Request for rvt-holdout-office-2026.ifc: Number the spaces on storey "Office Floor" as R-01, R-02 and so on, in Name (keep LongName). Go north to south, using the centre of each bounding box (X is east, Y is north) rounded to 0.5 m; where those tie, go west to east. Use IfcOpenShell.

First a look at what the model holds.

```python
import ifcopenshell
import ifcopenshell.util.element
import ifcopenshell.util.placement

model = ifcopenshell.open("rvt-holdout-office-2026.ifc")
print(model.schema)
storey = next(s for s in model.by_type("IfcBuildingStorey") if s.Name == "Office Floor")
spaces = [e for e in ifcopenshell.util.element.get_decomposition(storey) if e.is_a("IfcSpace")]
for e in sorted(spaces, key=lambda e: e.id()):
    origin = ifcopenshell.util.placement.get_local_placement(e.ObjectPlacement)[:3, 3]
    print(e.id(), e.Name, e.LongName, origin.round(2) + 0.0, sep=" | ")
```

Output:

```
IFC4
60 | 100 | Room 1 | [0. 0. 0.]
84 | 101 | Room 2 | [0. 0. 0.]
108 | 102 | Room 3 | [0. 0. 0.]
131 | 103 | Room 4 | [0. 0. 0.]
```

```python
import ifcopenshell
import ifcopenshell.geom
import ifcopenshell.util.element
import ifcopenshell.util.shape

model = ifcopenshell.open("rvt-holdout-office-2026.ifc")
settings = ifcopenshell.geom.settings()
settings.set("use-world-coords", True)


def centre(element):
    shape = ifcopenshell.geom.create_shape(settings, element)
    return ifcopenshell.util.shape.get_bbox_centroid(shape.geometry)


storey = next(s for s in model.by_type("IfcBuildingStorey") if s.Name == "Office Floor")
spaces = [e for e in ifcopenshell.util.element.get_decomposition(storey) if e.is_a("IfcSpace")]

# Insertion points can sit at a corner or the storey origin, so sort by the geometry (in metres).
centres = {e: centre(e) for e in spaces}
spaces.sort(key=lambda e: (-round(centres[e][1] / 0.5), centres[e][0]))

for i, e in enumerate(spaces, start=1):
    number = f"R-{i:02d}"
    e.Name = number
    print(e.id(), number)

model.write("rvt-holdout-office-2026-out.ifc")
```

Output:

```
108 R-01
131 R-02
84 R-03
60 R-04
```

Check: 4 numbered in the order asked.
